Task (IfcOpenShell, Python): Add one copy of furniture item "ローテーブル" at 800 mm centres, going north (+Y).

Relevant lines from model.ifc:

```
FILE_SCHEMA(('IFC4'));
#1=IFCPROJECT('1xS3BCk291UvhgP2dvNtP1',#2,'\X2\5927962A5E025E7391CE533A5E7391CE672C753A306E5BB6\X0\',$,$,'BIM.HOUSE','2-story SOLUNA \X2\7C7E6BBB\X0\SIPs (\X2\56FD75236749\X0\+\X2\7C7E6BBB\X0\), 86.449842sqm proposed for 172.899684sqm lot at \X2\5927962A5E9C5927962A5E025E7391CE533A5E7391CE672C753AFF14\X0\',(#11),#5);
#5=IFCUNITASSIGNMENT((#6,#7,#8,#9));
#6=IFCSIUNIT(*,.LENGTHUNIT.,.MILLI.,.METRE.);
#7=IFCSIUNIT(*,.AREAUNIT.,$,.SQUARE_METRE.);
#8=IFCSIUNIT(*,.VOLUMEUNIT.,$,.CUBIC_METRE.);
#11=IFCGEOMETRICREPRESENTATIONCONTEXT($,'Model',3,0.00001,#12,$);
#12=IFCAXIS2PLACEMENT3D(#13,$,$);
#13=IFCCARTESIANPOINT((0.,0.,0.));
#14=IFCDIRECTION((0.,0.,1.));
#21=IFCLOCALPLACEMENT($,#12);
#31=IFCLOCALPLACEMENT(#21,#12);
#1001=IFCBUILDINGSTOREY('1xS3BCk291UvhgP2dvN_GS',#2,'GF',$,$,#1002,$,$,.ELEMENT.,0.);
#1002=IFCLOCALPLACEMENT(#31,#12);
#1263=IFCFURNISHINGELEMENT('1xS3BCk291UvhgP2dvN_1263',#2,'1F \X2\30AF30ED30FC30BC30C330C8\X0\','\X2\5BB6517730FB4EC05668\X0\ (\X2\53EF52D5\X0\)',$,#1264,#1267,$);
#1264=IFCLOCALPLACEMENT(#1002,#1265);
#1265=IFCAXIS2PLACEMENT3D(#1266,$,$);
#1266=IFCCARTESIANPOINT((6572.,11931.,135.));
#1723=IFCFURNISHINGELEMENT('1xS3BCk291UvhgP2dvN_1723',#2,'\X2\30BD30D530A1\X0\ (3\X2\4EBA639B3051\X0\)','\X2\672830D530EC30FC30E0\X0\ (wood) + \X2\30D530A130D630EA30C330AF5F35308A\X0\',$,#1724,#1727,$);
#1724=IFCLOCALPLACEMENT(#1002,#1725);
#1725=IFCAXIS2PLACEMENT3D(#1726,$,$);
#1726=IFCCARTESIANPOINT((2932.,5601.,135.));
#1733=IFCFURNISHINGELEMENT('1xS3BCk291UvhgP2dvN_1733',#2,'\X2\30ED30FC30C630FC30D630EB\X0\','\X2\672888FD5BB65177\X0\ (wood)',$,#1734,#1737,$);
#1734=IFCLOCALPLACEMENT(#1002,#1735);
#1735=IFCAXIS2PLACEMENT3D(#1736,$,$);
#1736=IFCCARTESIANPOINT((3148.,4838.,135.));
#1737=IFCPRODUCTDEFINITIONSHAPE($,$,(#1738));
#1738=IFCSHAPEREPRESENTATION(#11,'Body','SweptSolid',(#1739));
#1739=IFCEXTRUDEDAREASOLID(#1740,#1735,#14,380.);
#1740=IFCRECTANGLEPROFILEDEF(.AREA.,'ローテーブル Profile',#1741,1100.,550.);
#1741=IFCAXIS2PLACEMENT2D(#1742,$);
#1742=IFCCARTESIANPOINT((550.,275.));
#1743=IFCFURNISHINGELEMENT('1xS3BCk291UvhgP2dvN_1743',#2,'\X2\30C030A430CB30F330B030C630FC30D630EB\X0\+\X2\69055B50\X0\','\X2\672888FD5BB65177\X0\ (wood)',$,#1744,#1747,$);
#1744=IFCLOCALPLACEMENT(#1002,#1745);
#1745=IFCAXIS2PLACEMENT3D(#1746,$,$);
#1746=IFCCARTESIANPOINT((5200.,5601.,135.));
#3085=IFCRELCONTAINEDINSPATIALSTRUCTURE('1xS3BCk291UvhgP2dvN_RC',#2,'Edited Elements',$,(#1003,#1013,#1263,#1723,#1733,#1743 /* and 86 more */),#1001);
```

```python
import numpy as np
import ifcopenshell
import ifcopenshell.api.geometry
import ifcopenshell.api.root
import ifcopenshell.util.element
import ifcopenshell.util.placement

model = ifcopenshell.open("model.ifc")


def reuse_history(source, copy):
    """copy_class also copies each property set's owner history, people and application; keep the originals."""
    for rel in copy.IsDefinedBy:
        if rel.is_a("IfcRelDefinesByProperties") and (history := rel.RelatingPropertyDefinition.OwnerHistory):
            rel.RelatingPropertyDefinition.OwnerHistory = source.OwnerHistory
            ifcopenshell.util.element.remove_deep2(model, history)


source = model.by_guid("1xS3BCk291UvhgP2dvN_1733")
base = ifcopenshell.util.placement.get_local_placement(source.ObjectPlacement)
step = np.array([0.0, 1.0, 0.0]) * 800.0

for i in range(1, 2):
    copy = ifcopenshell.api.root.copy_class(model, product=source)
    copy.Representation = ifcopenshell.util.element.copy_deep(
        model, source.Representation, exclude=["IfcGeometricRepresentationContext", "IfcRepresentationMap"]
    )
    reuse_history(source, copy)
    matrix = base.copy()
    matrix[:3, 3] += i * step
    print("added at", matrix[:3, 3].round(3) + 0.0)
    ifcopenshell.api.geometry.edit_object_placement(model, product=copy, matrix=matrix, is_si=False)

model.write("model-out.ifc")
```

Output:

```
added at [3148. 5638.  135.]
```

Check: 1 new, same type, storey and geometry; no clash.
